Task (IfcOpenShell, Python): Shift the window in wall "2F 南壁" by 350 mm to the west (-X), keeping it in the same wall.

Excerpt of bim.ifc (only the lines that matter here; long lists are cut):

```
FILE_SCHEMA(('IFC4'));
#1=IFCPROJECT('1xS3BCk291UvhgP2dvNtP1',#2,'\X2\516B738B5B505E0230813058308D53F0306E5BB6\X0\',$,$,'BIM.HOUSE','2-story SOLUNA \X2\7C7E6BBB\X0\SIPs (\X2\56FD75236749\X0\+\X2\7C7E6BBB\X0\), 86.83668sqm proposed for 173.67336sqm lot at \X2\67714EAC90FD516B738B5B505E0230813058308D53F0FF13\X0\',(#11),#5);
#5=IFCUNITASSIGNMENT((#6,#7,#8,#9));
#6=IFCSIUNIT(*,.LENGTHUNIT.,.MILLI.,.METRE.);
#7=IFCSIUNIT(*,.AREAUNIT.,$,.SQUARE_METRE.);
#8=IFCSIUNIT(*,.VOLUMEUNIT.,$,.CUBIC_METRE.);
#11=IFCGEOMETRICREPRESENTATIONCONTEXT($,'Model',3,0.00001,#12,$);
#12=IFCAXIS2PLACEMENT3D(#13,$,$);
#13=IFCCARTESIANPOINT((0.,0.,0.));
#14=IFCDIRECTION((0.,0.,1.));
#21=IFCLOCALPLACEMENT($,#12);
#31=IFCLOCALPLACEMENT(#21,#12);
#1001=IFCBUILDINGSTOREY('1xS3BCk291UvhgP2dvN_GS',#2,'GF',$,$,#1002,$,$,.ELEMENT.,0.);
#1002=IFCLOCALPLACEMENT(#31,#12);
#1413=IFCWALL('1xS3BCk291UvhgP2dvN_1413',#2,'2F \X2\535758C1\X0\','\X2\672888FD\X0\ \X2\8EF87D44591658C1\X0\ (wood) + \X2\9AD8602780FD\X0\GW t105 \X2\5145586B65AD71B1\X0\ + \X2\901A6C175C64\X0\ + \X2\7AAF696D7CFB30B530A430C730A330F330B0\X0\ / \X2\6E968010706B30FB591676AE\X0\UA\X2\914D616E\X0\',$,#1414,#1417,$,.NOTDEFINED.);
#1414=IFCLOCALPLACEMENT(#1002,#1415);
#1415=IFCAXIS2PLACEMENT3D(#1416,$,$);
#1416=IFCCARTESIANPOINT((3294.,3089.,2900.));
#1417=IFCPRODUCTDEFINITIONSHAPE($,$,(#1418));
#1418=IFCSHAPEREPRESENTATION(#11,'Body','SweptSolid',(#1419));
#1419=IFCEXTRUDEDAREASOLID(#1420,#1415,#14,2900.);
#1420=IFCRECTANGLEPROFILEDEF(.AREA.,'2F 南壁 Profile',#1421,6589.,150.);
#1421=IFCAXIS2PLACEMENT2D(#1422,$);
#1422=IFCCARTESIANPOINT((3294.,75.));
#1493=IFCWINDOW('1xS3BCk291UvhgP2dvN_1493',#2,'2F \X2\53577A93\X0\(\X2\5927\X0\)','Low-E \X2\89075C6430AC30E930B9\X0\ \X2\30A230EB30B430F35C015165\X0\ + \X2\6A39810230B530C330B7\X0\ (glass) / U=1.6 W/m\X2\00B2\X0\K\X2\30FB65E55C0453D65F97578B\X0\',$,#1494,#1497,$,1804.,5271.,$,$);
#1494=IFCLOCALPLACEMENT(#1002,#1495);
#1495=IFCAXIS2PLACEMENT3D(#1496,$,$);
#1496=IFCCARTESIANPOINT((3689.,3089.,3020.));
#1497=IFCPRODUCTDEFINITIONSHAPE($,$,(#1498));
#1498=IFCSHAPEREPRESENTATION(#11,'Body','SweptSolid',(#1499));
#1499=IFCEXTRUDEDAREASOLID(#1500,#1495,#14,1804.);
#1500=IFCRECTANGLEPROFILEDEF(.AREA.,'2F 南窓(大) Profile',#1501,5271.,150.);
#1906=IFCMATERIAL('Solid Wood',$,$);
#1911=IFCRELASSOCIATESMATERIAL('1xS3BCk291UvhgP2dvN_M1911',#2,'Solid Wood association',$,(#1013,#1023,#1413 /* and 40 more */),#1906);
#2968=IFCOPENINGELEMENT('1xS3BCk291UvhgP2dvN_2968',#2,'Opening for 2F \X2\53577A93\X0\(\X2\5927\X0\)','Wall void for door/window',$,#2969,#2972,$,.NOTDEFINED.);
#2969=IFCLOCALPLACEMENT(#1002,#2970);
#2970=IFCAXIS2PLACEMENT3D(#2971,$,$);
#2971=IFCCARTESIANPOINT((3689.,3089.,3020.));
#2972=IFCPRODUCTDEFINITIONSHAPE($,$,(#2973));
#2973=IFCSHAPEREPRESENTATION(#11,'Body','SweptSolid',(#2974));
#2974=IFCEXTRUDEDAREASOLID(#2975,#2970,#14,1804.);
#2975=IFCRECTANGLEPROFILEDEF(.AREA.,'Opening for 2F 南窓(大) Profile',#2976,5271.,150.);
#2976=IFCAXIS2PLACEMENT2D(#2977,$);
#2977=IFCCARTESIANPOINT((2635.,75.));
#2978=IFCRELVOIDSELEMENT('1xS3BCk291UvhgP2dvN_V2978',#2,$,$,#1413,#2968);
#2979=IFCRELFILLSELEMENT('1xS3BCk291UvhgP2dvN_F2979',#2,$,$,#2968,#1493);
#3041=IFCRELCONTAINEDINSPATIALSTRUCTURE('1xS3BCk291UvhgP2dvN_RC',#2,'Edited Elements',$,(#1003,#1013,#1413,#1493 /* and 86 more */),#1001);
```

```python
import ifcopenshell
import ifcopenshell.api.geometry
import ifcopenshell.util.placement

model = ifcopenshell.open("bim.ifc")

window = model.by_guid("1xS3BCk291UvhgP2dvN_1493")
opening = window.FillsVoids[0].RelatingOpeningElement
wall = opening.VoidsElements[0].RelatingBuildingElement

wall_matrix = ifcopenshell.util.placement.get_local_placement(wall.ObjectPlacement)
shift = wall_matrix[:3, 0] * -350.0
before = ifcopenshell.util.placement.get_local_placement(window.ObjectPlacement)[:3, 3].copy()

# The window is not placed relative to its opening, so move both.
for product in (opening, window):
    matrix = ifcopenshell.util.placement.get_local_placement(product.ObjectPlacement)
    matrix[:3, 3] += shift
    ifcopenshell.api.geometry.edit_object_placement(model, product=product, matrix=matrix, is_si=False)

after = ifcopenshell.util.placement.get_local_placement(window.ObjectPlacement)[:3, 3]
print("window moved by", (after - before).round(3) + 0.0)

model.write("bim-out.ifc")
```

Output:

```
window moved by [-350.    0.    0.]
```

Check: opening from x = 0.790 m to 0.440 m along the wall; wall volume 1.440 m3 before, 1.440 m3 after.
